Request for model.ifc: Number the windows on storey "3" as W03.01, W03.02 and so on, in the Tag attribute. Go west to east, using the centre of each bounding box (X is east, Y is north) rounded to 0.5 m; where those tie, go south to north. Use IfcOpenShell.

First a look at what the model holds.

```python
import ifcopenshell
import ifcopenshell.util.element
import ifcopenshell.util.placement

model = ifcopenshell.open("model.ifc")
print(model.schema)
storey = next(s for s in model.by_type("IfcBuildingStorey") if s.Name == "3")
windows = [e for e in ifcopenshell.util.element.get_decomposition(storey) if e.is_a("IfcWindow")]
for e in sorted(windows, key=lambda e: e.id()):
    origin = ifcopenshell.util.placement.get_local_placement(e.ObjectPlacement)[:3, 3]
    print(e.id(), e.Tag, e.Name, origin.round(2) + 0.0, sep=" | ")
```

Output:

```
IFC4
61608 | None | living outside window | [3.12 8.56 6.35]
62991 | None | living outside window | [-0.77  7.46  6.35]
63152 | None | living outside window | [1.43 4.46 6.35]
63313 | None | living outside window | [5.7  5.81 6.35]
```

```python
import ifcopenshell
import ifcopenshell.geom
import ifcopenshell.util.element
import ifcopenshell.util.shape

model = ifcopenshell.open("model.ifc")
settings = ifcopenshell.geom.settings()
settings.set("use-world-coords", True)


def centre(element):
    shape = ifcopenshell.geom.create_shape(settings, element)
    return ifcopenshell.util.shape.get_bbox_centroid(shape.geometry)


storey = next(s for s in model.by_type("IfcBuildingStorey") if s.Name == "3")
windows = [e for e in ifcopenshell.util.element.get_decomposition(storey) if e.is_a("IfcWindow")]

# Insertion points can sit at a corner or the storey origin, so sort by the geometry (in metres).
centres = {e: centre(e) for e in windows}
windows.sort(key=lambda e: (round(centres[e][0] / 0.5), centres[e][1]))

for i, e in enumerate(windows, start=1):
    number = f"W03.{i:02d}"
    e.Tag = number
    print(e.id(), number)

model.write("model_edited.ifc")
```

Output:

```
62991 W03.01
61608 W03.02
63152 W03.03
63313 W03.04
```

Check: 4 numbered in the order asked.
